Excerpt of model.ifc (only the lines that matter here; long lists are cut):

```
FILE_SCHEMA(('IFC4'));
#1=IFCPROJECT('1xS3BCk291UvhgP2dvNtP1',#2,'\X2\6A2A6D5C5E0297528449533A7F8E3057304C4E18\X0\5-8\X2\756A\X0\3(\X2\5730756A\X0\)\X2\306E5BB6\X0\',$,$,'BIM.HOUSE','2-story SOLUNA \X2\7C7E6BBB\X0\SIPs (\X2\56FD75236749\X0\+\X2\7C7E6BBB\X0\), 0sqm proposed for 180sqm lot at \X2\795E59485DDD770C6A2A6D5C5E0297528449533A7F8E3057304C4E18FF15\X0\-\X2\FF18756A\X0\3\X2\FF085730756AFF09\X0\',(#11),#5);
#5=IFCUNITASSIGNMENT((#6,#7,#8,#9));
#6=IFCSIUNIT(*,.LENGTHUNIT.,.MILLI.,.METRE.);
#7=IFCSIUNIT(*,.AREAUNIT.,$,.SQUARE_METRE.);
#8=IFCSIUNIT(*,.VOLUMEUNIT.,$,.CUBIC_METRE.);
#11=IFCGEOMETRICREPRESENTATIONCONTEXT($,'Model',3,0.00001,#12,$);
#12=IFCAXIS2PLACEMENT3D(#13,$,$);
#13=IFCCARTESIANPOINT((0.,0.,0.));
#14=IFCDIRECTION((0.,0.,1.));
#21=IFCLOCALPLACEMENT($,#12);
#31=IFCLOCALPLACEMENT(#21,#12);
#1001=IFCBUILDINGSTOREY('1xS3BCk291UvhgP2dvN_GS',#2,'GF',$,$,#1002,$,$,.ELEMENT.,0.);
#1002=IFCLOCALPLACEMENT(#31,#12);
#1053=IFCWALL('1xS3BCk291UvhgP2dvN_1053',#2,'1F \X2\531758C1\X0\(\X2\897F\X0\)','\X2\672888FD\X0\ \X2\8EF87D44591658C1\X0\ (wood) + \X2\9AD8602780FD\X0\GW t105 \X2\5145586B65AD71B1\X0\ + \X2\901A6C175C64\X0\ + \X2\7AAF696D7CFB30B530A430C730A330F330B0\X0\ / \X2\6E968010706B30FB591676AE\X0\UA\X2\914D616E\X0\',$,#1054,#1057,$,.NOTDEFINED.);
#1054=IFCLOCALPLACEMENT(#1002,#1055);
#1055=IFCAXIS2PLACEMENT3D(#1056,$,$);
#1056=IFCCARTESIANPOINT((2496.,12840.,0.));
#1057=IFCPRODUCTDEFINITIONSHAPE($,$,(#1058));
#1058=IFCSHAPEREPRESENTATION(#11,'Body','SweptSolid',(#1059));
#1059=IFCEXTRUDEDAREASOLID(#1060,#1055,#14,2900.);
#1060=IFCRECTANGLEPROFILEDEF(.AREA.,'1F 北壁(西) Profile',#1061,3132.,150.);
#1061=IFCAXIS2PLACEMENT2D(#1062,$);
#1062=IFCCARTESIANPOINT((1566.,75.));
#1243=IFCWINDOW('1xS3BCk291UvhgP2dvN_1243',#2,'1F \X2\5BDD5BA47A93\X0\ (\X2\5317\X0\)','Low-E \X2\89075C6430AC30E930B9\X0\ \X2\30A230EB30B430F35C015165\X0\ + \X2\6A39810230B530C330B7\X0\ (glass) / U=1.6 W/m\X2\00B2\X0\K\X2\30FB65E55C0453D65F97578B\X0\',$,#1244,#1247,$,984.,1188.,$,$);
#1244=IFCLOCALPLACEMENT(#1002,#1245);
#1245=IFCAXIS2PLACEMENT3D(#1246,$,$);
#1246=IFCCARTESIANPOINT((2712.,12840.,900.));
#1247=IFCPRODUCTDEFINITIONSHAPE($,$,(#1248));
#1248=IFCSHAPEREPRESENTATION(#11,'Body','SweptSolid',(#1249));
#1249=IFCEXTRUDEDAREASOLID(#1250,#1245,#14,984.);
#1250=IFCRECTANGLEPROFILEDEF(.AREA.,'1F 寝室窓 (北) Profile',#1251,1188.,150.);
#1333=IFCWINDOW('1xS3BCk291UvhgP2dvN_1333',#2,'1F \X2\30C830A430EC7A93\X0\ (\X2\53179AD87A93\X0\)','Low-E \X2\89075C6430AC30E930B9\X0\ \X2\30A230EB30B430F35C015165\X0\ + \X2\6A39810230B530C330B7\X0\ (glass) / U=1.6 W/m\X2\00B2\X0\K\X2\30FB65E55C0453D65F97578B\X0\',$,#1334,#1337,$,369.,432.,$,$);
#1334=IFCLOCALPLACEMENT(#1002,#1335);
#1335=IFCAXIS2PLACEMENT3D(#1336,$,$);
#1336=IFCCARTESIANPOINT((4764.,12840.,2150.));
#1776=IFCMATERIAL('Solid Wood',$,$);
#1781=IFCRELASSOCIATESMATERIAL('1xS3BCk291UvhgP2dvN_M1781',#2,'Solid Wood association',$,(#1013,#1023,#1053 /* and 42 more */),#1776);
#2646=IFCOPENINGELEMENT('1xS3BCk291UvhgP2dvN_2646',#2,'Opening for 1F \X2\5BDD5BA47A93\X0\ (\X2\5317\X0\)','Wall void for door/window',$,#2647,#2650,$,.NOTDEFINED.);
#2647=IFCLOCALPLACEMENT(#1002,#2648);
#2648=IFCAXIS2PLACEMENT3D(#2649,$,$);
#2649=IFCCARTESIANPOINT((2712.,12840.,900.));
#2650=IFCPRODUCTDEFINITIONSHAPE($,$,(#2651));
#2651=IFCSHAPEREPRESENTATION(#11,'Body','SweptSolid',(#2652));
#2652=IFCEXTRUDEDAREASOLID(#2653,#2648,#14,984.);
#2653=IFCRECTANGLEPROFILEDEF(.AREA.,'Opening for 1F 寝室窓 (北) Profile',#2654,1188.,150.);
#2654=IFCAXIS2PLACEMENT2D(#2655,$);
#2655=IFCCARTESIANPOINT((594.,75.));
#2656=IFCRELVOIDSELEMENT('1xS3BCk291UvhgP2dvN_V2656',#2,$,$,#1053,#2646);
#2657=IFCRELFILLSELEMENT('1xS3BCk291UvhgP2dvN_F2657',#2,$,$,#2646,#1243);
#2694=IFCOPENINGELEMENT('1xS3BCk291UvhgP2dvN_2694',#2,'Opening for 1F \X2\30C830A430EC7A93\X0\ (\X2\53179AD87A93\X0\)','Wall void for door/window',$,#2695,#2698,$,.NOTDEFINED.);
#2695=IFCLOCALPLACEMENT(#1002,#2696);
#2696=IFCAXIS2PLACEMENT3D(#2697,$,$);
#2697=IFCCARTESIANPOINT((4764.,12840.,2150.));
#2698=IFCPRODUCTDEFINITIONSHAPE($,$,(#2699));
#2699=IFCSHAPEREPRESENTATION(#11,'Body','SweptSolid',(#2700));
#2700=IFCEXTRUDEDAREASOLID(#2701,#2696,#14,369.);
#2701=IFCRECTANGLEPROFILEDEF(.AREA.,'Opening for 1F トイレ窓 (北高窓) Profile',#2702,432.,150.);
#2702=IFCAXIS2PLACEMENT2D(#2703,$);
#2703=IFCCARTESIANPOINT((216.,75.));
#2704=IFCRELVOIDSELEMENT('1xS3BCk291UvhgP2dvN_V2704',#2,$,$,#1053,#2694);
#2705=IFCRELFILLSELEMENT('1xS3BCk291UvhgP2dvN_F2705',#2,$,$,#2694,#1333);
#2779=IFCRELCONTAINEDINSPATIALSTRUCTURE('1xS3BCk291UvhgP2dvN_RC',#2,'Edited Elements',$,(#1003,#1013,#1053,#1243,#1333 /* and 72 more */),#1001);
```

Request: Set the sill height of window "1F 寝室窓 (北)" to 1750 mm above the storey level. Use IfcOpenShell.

```python
import numpy as np
import ifcopenshell
import ifcopenshell.api.geometry
import ifcopenshell.geom
import ifcopenshell.util.element
import ifcopenshell.util.placement
import ifcopenshell.util.shape
import ifcopenshell.util.unit

model = ifcopenshell.open("model.ifc")
unit_scale = ifcopenshell.util.unit.calculate_unit_scale(model)

window = model.by_guid("1xS3BCk291UvhgP2dvN_1243")
opening = window.FillsVoids[0].RelatingOpeningElement
storey = ifcopenshell.util.element.get_container(window, ifc_class="IfcBuildingStorey")
level = ifcopenshell.util.placement.get_local_placement(storey.ObjectPlacement)[2, 3]

# The opening's origin need not be at the sill, so measure its lowest point.
shape = ifcopenshell.geom.create_shape(ifcopenshell.geom.settings(), opening)
bottom = ifcopenshell.util.shape.get_shape_bottom_elevation(shape, shape.geometry) / unit_scale
dz = level + 1.75 / unit_scale - bottom

shift = np.array([0.0, 0.0, dz])
# The window is not placed relative to its opening, so move both.
for product in (opening, window):
    matrix = ifcopenshell.util.placement.get_local_placement(product.ObjectPlacement)
    matrix[:3, 3] += shift
    ifcopenshell.api.geometry.edit_object_placement(model, product=product, matrix=matrix, is_si=False)

print(f"moved by {dz * unit_scale:+.3f} m")

model.write("model_v2.ifc")
```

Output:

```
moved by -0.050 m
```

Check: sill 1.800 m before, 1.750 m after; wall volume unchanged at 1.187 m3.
